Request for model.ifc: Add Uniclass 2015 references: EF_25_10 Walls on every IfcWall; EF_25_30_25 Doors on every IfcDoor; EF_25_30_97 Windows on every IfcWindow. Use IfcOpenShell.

First a look at what the model holds.

```python
import ifcopenshell

model = ifcopenshell.open("model.ifc")
print(model.schema)
print("classifications:", [c.Name for c in model.by_type("IfcClassification")])
for ifc_class in ("IfcDoor", "IfcRoof", "IfcStair", "IfcWall", "IfcWindow"):
    print(ifc_class, len(model.by_type(ifc_class)))
```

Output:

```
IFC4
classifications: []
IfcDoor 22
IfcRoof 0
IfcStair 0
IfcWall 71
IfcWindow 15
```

```python
import ifcopenshell
import ifcopenshell.api.classification

model = ifcopenshell.open("model.ifc")

system = ifcopenshell.api.classification.add_classification(model, classification="Uniclass 2015")

codes = {
    "IfcWall": ("EF_25_10", "Walls"),
    "IfcDoor": ("EF_25_30_25", "Doors"),
    "IfcWindow": ("EF_25_30_97", "Windows"),
}
for ifc_class, (code, name) in codes.items():
    products = model.by_type(ifc_class)
    ifcopenshell.api.classification.add_reference(
        model, products=products, classification=system, identification=code, name=name
    )
    print(code, len(products))

model.write("model_edited.ifc")
```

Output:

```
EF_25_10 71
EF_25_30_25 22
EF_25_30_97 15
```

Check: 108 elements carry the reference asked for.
